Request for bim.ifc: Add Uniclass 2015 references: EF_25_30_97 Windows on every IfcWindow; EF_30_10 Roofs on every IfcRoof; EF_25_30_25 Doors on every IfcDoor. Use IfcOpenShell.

First a look at what the model holds.

```python
import ifcopenshell

model = ifcopenshell.open("bim.ifc")
print(model.schema)
print("classifications:", [c.Name for c in model.by_type("IfcClassification")])
for ifc_class in ("IfcDoor", "IfcRoof", "IfcStair", "IfcWall", "IfcWindow"):
    print(ifc_class, len(model.by_type(ifc_class)))
```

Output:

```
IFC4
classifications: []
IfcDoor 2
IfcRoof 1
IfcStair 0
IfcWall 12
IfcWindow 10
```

```python
import ifcopenshell
import ifcopenshell.api.classification

model = ifcopenshell.open("bim.ifc")

system = ifcopenshell.api.classification.add_classification(model, classification="Uniclass 2015")

codes = {
    "IfcWindow": ("EF_25_30_97", "Windows"),
    "IfcRoof": ("EF_30_10", "Roofs"),
    "IfcDoor": ("EF_25_30_25", "Doors"),
}
for ifc_class, (code, name) in codes.items():
    products = model.by_type(ifc_class)
    ifcopenshell.api.classification.add_reference(
        model, products=products, classification=system, identification=code, name=name
    )
    print(code, len(products))

model.write("bim-out.ifc")
```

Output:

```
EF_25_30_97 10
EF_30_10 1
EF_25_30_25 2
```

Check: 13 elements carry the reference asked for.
